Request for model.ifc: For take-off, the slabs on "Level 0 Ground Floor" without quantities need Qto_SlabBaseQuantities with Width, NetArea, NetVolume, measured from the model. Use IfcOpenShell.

First a look at what the model holds.

```python
import ifcopenshell
import ifcopenshell.util.element
import ifcopenshell.util.unit

model = ifcopenshell.open("model.ifc")
print(model.schema)
for unit_type in ("LENGTHUNIT", "AREAUNIT", "VOLUMEUNIT"):
    print(unit_type, ifcopenshell.util.unit.calculate_unit_scale(model, unit_type))
storey = next(s for s in model.by_type("IfcBuildingStorey") if s.Name == "Level 0 Ground Floor")
slabs = [e for e in ifcopenshell.util.element.get_decomposition(storey) if e.is_a("IfcSlab")]
for e in sorted(slabs, key=lambda e: e.id()):
    print(e.id(), e.is_a(), e.Name, list(ifcopenshell.util.element.get_psets(e, qtos_only=True)), sep=" | ")
```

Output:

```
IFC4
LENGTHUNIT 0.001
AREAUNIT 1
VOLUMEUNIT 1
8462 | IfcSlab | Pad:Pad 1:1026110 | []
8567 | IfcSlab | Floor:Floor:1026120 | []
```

```python
import ifcopenshell
import ifcopenshell.api.pset
import ifcopenshell.geom
import ifcopenshell.util.element
import ifcopenshell.util.shape
import ifcopenshell.util.unit

model = ifcopenshell.open("model.ifc")
unit_scale = ifcopenshell.util.unit.calculate_unit_scale(model)
area_scale = ifcopenshell.util.unit.calculate_unit_scale(model, "AREAUNIT")
volume_scale = ifcopenshell.util.unit.calculate_unit_scale(model, "VOLUMEUNIT")
settings = ifcopenshell.geom.settings()

storey = next(s for s in model.by_type("IfcBuildingStorey") if s.Name == "Level 0 Ground Floor")
slabs = [e for e in ifcopenshell.util.element.get_decomposition(storey) if e.is_a("IfcSlab")]

for e in sorted(slabs, key=lambda e: e.id()):
    if ifcopenshell.util.element.get_psets(e, qtos_only=True, should_inherit=False):
        continue
    # Geometry comes back in metres, in the element's own axes.
    shape = ifcopenshell.geom.create_shape(settings, e)
    values = {
        "Width": ifcopenshell.util.shape.get_z(shape.geometry) / unit_scale,
        "NetArea": ifcopenshell.util.shape.get_footprint_area(shape.geometry) / area_scale,
        "NetVolume": ifcopenshell.util.shape.get_volume(shape.geometry) / volume_scale,
    }
    qto = ifcopenshell.api.pset.add_qto(model, product=e, name="Qto_SlabBaseQuantities")
    ifcopenshell.api.pset.edit_qto(model, qto=qto, properties=values)
    print(e.id(), {k: round(v, 3) for k, v in values.items()})

model.write("model_updated.ifc")
```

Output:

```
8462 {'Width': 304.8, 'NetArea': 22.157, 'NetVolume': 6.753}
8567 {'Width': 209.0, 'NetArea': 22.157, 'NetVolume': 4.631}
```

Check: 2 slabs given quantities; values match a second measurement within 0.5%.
